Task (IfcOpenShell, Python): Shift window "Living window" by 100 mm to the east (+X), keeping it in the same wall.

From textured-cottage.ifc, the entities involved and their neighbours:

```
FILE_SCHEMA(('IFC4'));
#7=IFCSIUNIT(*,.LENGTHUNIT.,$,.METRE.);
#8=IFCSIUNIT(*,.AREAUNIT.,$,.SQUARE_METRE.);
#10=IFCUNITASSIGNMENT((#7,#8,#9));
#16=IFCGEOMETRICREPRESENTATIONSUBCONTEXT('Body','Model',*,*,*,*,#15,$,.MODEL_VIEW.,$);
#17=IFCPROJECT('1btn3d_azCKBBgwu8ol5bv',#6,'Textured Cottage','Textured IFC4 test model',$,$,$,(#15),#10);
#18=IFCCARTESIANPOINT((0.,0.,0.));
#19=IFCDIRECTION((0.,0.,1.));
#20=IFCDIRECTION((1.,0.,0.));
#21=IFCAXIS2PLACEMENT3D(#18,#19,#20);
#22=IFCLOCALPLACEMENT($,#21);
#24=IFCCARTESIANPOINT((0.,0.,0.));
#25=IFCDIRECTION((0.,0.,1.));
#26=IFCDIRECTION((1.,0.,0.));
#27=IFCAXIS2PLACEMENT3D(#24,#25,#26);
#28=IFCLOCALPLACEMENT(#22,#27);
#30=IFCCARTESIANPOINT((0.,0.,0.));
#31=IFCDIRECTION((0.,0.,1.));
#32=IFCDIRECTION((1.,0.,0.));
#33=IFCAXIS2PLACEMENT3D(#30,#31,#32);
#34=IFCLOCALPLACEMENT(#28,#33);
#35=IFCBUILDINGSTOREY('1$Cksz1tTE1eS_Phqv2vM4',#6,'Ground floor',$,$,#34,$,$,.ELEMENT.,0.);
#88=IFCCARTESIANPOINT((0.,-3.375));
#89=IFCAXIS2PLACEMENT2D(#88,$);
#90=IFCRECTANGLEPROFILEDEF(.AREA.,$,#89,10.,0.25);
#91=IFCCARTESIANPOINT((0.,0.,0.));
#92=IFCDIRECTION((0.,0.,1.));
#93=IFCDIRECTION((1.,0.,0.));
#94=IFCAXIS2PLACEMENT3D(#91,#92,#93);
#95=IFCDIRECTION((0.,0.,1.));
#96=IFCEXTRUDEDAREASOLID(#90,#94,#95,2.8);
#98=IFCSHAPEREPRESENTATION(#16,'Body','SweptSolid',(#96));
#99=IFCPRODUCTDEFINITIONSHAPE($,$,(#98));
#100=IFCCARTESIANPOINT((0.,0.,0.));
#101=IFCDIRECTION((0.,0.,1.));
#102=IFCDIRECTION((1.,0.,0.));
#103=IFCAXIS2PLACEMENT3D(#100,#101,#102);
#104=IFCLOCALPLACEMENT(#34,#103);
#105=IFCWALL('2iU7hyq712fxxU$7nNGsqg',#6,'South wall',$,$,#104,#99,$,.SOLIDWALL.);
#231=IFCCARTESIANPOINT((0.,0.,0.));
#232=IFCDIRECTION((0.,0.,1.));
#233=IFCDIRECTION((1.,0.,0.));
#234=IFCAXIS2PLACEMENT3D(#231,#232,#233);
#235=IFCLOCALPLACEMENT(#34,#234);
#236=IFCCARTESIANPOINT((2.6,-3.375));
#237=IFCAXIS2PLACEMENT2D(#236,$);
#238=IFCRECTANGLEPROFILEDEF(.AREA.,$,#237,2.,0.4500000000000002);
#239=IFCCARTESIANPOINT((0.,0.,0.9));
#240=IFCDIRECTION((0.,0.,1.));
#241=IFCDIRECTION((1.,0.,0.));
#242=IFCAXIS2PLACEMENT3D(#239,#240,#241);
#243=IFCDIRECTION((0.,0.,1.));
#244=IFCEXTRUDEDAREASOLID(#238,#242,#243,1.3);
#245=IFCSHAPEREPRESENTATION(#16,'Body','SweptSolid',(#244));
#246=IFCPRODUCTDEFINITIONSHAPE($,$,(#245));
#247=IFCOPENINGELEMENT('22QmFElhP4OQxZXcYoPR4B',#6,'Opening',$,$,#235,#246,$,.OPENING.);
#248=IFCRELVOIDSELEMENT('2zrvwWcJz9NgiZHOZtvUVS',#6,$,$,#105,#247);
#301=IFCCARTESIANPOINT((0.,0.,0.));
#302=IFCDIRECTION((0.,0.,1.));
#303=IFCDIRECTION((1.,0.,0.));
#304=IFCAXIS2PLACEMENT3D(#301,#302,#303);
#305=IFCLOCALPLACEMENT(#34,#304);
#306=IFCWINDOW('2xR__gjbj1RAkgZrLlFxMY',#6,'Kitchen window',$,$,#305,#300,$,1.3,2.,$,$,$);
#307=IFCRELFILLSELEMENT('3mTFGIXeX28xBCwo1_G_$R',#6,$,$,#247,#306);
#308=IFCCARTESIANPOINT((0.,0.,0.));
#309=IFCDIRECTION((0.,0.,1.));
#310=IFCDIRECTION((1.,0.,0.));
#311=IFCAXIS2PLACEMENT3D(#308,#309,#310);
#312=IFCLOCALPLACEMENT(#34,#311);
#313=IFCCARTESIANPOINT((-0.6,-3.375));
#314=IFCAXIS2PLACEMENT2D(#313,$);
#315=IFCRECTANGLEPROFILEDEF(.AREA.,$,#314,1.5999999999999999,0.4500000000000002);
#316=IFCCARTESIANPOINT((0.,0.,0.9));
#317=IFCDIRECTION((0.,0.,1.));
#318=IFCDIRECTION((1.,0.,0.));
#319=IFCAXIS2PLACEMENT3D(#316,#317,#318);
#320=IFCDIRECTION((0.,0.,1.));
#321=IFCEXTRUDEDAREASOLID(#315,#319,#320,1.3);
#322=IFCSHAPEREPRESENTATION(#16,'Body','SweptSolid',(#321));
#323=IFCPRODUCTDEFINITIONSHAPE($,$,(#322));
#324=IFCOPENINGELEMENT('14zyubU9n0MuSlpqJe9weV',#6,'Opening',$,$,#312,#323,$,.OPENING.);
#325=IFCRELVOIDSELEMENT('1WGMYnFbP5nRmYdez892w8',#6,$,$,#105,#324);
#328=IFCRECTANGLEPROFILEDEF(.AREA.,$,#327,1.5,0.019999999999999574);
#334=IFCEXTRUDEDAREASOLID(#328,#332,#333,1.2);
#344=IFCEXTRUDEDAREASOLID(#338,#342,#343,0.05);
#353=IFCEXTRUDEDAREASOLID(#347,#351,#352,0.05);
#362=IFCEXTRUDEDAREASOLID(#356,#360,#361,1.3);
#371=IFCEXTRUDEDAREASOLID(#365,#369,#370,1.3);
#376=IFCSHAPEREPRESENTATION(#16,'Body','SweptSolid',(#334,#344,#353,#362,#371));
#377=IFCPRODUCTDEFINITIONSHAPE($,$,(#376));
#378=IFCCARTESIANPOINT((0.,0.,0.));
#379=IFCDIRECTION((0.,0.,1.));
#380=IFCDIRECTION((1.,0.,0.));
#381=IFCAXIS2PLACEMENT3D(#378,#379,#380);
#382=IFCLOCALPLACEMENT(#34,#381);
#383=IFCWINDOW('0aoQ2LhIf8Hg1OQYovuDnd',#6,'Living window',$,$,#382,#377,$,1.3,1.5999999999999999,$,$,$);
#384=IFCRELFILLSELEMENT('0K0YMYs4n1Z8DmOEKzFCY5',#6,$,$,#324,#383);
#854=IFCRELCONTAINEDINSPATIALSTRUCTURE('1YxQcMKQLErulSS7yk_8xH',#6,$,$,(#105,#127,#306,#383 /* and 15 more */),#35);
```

```python
import ifcopenshell
import ifcopenshell.api.geometry
import ifcopenshell.util.placement
import ifcopenshell.util.unit

model = ifcopenshell.open("textured-cottage.ifc")
unit_scale = ifcopenshell.util.unit.calculate_unit_scale(model)

window = model.by_guid("0aoQ2LhIf8Hg1OQYovuDnd")
opening = window.FillsVoids[0].RelatingOpeningElement
wall = opening.VoidsElements[0].RelatingBuildingElement

wall_matrix = ifcopenshell.util.placement.get_local_placement(wall.ObjectPlacement)
shift = wall_matrix[:3, 0] * 0.1 / unit_scale
before = ifcopenshell.util.placement.get_local_placement(window.ObjectPlacement)[:3, 3].copy()

# The window is not placed relative to its opening, so move both.
for product in (opening, window):
    matrix = ifcopenshell.util.placement.get_local_placement(product.ObjectPlacement)
    matrix[:3, 3] += shift
    ifcopenshell.api.geometry.edit_object_placement(model, product=product, matrix=matrix, is_si=False)

after = ifcopenshell.util.placement.get_local_placement(window.ObjectPlacement)[:3, 3]
print("window moved by", (after - before).round(3) + 0.0)

model.write("textured-cottage-out.ifc")
```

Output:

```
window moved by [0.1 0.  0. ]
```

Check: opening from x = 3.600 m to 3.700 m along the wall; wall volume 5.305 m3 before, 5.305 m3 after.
